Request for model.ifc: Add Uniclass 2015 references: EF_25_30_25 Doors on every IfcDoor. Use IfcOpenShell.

First a look at what the model holds.

```python
import ifcopenshell

model = ifcopenshell.open("model.ifc")
print(model.schema)
print("classifications:", [c.Name for c in model.by_type("IfcClassification")])
for ifc_class in ("IfcDoor", "IfcRoof", "IfcStair", "IfcWall", "IfcWindow"):
    print(ifc_class, len(model.by_type(ifc_class)))
```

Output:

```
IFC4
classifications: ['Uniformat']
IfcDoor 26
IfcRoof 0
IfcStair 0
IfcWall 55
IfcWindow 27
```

```python
import ifcopenshell
import ifcopenshell.api.classification

model = ifcopenshell.open("model.ifc")

system = ifcopenshell.api.classification.add_classification(model, classification="Uniclass 2015")

codes = {
    "IfcDoor": ("EF_25_30_25", "Doors"),
}
for ifc_class, (code, name) in codes.items():
    products = model.by_type(ifc_class)
    ifcopenshell.api.classification.add_reference(
        model, products=products, classification=system, identification=code, name=name
    )
    print(code, len(products))

model.write("model_rev.ifc")
```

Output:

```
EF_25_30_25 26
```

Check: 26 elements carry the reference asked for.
